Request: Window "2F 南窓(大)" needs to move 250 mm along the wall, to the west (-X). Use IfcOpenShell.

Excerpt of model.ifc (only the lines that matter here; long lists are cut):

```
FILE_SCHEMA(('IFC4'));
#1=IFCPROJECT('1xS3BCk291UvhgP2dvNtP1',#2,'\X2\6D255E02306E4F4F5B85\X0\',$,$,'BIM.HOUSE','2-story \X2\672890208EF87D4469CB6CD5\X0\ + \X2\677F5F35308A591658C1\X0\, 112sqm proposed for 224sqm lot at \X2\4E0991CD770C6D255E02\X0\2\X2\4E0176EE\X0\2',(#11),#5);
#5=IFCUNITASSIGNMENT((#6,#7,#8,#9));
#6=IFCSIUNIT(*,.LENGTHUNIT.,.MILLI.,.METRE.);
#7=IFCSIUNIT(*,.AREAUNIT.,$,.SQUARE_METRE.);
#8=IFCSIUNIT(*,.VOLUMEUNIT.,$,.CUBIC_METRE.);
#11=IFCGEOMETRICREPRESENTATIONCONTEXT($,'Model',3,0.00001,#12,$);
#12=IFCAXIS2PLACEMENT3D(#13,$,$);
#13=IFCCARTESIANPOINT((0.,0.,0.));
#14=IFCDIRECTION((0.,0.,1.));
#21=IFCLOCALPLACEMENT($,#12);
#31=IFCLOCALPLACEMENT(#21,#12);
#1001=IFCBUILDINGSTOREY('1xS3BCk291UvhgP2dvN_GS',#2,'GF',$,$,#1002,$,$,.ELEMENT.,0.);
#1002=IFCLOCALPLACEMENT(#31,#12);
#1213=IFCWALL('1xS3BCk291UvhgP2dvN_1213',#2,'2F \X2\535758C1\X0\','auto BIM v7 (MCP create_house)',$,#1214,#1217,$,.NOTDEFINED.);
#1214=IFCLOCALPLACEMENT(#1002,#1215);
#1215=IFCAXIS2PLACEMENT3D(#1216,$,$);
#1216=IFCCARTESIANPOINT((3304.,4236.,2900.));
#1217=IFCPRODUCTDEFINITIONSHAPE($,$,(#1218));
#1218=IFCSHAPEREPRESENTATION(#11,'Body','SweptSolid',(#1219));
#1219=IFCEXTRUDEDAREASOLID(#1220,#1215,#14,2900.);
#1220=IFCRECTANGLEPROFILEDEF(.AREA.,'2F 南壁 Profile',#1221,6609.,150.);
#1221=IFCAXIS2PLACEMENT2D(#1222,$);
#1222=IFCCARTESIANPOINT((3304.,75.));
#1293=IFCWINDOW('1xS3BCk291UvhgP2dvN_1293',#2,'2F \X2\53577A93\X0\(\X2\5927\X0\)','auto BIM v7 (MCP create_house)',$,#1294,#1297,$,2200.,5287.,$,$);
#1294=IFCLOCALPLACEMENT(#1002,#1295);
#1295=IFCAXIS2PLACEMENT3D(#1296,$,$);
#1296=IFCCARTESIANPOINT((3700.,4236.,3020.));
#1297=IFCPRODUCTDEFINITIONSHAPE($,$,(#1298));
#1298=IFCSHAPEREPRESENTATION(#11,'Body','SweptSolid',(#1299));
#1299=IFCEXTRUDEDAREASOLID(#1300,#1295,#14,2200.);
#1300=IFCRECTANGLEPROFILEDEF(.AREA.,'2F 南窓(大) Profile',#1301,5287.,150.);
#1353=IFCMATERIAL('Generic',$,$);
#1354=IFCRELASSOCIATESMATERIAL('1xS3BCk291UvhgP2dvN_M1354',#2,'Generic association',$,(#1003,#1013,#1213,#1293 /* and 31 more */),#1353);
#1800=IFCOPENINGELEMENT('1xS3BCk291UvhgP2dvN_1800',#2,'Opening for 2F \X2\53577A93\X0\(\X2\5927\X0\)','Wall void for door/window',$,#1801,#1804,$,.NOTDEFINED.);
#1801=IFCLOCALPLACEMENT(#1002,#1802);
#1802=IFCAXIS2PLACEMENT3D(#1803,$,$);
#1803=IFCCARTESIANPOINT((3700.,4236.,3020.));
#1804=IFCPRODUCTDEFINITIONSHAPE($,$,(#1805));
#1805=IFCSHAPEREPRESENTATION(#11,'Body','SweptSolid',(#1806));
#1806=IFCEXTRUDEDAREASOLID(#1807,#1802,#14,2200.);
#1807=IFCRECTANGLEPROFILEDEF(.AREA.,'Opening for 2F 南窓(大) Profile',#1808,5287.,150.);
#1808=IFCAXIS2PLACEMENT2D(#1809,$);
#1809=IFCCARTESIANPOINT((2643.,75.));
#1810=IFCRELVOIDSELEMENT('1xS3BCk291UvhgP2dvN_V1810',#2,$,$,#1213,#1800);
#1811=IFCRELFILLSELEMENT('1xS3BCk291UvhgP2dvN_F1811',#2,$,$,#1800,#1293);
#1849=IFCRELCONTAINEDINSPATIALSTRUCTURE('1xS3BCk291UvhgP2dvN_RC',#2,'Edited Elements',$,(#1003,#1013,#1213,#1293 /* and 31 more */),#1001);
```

```python
import ifcopenshell
import ifcopenshell.api.geometry
import ifcopenshell.util.placement

model = ifcopenshell.open("model.ifc")

window = model.by_guid("1xS3BCk291UvhgP2dvN_1293")
opening = window.FillsVoids[0].RelatingOpeningElement
wall = opening.VoidsElements[0].RelatingBuildingElement

wall_matrix = ifcopenshell.util.placement.get_local_placement(wall.ObjectPlacement)
shift = wall_matrix[:3, 0] * -250.0
before = ifcopenshell.util.placement.get_local_placement(window.ObjectPlacement)[:3, 3].copy()

# The window is not placed relative to its opening, so move both.
for product in (opening, window):
    matrix = ifcopenshell.util.placement.get_local_placement(product.ObjectPlacement)
    matrix[:3, 3] += shift
    ifcopenshell.api.geometry.edit_object_placement(model, product=product, matrix=matrix, is_si=False)

after = ifcopenshell.util.placement.get_local_placement(window.ObjectPlacement)[:3, 3]
print("window moved by", (after - before).round(3) + 0.0)

model.write("model_v2.ifc")
```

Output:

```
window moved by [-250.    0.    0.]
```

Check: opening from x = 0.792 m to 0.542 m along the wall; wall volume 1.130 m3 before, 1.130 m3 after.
